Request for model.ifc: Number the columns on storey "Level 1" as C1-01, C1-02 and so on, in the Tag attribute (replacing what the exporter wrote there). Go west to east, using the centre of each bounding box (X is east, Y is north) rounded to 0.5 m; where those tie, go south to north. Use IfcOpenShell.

First a look at what the model holds.

```python
import ifcopenshell
import ifcopenshell.util.element
import ifcopenshell.util.placement

model = ifcopenshell.open("model.ifc")
print(model.schema)
storey = next(s for s in model.by_type("IfcBuildingStorey") if s.Name == "Level 1")
columns = [e for e in ifcopenshell.util.element.get_decomposition(storey) if e.is_a("IfcColumn")]
for e in sorted(columns, key=lambda e: e.id()):
    origin = ifcopenshell.util.placement.get_local_placement(e.ObjectPlacement)[:3, 3]
    print(e.id(), e.Tag, e.Name, origin.round(2) + 0.0, sep=" | ")
```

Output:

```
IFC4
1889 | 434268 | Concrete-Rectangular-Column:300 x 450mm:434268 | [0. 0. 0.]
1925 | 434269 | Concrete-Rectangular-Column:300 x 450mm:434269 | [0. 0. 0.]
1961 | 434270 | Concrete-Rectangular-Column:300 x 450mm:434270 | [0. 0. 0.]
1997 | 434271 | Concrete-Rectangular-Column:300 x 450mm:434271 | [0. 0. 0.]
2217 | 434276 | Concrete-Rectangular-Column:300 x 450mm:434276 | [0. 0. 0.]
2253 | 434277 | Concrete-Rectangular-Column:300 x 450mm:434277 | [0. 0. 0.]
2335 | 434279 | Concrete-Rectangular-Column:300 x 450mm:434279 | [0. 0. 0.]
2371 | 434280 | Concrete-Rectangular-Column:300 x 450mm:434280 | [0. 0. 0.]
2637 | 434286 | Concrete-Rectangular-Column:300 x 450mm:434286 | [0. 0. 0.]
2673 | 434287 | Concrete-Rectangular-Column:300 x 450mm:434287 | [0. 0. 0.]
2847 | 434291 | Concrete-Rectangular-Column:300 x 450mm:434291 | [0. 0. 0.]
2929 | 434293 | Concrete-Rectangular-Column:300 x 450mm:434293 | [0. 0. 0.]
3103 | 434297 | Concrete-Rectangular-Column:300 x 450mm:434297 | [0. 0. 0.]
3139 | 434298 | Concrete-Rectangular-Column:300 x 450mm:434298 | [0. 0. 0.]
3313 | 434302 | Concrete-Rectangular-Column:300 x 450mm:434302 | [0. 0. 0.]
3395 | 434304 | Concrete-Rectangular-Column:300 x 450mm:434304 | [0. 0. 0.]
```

```python
import ifcopenshell
import ifcopenshell.geom
import ifcopenshell.util.element
import ifcopenshell.util.shape

model = ifcopenshell.open("model.ifc")
settings = ifcopenshell.geom.settings()
settings.set("use-world-coords", True)


def centre(element):
    shape = ifcopenshell.geom.create_shape(settings, element)
    return ifcopenshell.util.shape.get_bbox_centroid(shape.geometry)


storey = next(s for s in model.by_type("IfcBuildingStorey") if s.Name == "Level 1")
columns = [e for e in ifcopenshell.util.element.get_decomposition(storey) if e.is_a("IfcColumn")]

# Insertion points can sit at a corner or the storey origin, so sort by the geometry (in metres).
centres = {e: centre(e) for e in columns}
columns.sort(key=lambda e: (round(centres[e][0] / 0.5), centres[e][1]))

for i, e in enumerate(columns, start=1):
    number = f"C1-{i:02d}"
    e.Tag = number
    print(e.id(), number)

model.write("model_updated.ifc")
```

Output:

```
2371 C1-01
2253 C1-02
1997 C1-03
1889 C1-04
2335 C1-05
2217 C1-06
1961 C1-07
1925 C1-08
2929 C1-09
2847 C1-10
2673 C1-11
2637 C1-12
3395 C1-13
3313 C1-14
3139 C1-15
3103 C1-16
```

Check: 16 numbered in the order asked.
